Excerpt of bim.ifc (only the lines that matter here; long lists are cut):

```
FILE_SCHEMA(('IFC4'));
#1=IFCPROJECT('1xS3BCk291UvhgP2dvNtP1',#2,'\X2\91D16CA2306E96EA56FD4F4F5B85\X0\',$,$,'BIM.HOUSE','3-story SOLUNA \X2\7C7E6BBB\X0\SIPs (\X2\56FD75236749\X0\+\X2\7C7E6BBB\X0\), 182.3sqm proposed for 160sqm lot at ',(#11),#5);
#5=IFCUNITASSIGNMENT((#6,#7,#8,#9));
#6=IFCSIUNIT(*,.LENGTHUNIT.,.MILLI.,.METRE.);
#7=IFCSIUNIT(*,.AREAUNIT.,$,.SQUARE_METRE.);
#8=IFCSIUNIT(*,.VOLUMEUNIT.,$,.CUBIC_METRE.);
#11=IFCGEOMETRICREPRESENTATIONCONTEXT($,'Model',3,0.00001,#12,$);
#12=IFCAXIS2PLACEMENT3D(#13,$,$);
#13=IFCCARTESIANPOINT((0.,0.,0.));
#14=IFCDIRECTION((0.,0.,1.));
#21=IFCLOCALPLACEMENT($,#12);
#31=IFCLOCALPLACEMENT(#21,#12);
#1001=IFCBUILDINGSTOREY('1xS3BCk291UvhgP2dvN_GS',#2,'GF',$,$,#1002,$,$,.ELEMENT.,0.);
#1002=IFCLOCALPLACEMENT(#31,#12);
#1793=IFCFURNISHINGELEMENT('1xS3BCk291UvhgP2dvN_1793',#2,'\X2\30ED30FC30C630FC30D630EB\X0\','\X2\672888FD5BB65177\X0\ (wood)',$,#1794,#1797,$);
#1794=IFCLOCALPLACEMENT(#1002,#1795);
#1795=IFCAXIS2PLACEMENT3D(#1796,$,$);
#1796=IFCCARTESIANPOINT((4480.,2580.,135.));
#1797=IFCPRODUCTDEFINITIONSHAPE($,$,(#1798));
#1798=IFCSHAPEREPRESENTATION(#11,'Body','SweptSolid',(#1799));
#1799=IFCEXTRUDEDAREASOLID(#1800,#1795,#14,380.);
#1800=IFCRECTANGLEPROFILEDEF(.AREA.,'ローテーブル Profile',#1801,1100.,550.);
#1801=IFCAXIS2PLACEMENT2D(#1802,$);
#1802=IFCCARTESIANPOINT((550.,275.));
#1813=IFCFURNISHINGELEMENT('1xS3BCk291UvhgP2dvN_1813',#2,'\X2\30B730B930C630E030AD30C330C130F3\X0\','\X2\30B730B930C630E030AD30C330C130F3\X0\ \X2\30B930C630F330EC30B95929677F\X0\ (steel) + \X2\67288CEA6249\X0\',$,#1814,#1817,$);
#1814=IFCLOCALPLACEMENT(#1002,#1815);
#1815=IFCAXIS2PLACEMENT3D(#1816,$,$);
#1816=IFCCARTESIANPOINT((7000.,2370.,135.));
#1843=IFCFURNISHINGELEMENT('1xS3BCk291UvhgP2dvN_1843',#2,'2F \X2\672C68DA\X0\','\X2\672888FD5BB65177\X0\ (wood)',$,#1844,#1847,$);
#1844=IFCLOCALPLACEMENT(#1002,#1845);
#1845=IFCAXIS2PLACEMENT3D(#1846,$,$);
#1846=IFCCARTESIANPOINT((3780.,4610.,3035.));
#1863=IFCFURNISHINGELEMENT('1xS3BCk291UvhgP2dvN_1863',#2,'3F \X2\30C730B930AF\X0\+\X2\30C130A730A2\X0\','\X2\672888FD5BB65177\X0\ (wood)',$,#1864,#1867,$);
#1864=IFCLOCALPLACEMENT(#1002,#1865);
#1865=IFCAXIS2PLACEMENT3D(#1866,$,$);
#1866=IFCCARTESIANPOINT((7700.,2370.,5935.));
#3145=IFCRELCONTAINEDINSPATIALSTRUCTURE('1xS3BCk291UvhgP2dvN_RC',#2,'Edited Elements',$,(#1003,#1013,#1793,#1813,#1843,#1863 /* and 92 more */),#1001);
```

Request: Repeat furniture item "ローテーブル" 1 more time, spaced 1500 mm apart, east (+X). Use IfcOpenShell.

```python
import numpy as np
import ifcopenshell
import ifcopenshell.api.geometry
import ifcopenshell.api.root
import ifcopenshell.util.element
import ifcopenshell.util.placement

model = ifcopenshell.open("bim.ifc")


def reuse_history(source, copy):
    """copy_class also copies each property set's owner history, people and application; keep the originals."""
    for rel in copy.IsDefinedBy:
        if rel.is_a("IfcRelDefinesByProperties") and (history := rel.RelatingPropertyDefinition.OwnerHistory):
            rel.RelatingPropertyDefinition.OwnerHistory = source.OwnerHistory
            ifcopenshell.util.element.remove_deep2(model, history)


source = model.by_guid("1xS3BCk291UvhgP2dvN_1793")
base = ifcopenshell.util.placement.get_local_placement(source.ObjectPlacement)
step = np.array([1.0, 0.0, 0.0]) * 1500.0

for i in range(1, 2):
    copy = ifcopenshell.api.root.copy_class(model, product=source)
    copy.Representation = ifcopenshell.util.element.copy_deep(
        model, source.Representation, exclude=["IfcGeometricRepresentationContext", "IfcRepresentationMap"]
    )
    reuse_history(source, copy)
    matrix = base.copy()
    matrix[:3, 3] += i * step
    print("added at", matrix[:3, 3].round(3) + 0.0)
    ifcopenshell.api.geometry.edit_object_placement(model, product=copy, matrix=matrix, is_si=False)

model.write("bim_updated.ifc")
```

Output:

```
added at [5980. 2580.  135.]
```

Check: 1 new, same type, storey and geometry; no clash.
